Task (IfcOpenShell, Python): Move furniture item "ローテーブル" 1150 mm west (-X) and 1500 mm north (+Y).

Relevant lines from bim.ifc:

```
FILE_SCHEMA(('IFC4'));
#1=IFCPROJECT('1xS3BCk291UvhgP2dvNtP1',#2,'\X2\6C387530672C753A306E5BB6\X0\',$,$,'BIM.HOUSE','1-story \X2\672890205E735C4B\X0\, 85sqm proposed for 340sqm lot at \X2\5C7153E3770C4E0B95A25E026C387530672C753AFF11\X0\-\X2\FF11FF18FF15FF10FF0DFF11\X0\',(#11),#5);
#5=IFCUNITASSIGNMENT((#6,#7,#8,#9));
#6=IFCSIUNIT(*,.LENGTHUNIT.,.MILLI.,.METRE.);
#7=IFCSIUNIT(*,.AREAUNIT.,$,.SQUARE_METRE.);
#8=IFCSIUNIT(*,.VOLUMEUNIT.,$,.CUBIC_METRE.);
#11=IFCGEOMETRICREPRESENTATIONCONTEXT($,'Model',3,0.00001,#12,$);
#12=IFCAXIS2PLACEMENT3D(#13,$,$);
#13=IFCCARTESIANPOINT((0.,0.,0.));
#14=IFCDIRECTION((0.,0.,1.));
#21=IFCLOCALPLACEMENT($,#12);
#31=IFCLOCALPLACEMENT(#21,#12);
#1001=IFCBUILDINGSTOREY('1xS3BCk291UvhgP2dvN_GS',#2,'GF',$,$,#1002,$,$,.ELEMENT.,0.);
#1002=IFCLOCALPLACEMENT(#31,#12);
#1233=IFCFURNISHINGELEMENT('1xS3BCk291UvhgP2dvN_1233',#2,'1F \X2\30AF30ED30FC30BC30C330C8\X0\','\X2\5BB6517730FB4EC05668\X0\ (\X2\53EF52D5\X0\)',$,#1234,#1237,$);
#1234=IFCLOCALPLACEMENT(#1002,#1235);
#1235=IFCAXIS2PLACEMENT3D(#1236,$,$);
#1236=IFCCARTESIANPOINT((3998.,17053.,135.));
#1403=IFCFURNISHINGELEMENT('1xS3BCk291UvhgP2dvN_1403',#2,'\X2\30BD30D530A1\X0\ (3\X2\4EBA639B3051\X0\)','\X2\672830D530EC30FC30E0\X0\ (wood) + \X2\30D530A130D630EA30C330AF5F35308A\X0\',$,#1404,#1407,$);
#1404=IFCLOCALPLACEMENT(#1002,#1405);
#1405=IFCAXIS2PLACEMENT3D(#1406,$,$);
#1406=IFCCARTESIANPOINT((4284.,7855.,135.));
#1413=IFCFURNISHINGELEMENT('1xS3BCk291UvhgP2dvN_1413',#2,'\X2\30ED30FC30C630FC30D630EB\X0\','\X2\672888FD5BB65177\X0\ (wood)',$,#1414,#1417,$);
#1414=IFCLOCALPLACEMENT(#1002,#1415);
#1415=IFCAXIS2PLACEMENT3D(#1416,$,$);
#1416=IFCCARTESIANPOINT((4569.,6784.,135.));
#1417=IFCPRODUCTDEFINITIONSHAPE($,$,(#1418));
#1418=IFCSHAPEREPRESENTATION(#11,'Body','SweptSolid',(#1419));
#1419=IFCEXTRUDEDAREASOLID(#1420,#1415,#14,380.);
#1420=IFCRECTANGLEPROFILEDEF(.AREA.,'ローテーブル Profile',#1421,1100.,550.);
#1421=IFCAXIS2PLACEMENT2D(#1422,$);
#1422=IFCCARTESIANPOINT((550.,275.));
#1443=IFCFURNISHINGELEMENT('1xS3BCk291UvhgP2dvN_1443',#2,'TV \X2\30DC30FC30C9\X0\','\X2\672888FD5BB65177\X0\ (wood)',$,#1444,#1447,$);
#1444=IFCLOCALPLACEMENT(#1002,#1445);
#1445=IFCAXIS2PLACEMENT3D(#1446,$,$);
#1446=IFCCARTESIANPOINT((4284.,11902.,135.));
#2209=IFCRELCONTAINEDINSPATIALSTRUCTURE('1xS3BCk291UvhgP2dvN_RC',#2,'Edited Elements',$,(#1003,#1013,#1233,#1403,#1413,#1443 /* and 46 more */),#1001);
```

```python
import ifcopenshell
import ifcopenshell.api.geometry
import ifcopenshell.util.placement
import ifcopenshell.util.unit

model = ifcopenshell.open("bim.ifc")
unit_scale = ifcopenshell.util.unit.calculate_unit_scale(model)

item = model.by_guid("1xS3BCk291UvhgP2dvN_1413")
matrix = ifcopenshell.util.placement.get_local_placement(item.ObjectPlacement)
matrix[0, 3] -= 1.15 / unit_scale
matrix[1, 3] += 1.5 / unit_scale
ifcopenshell.api.geometry.edit_object_placement(model, product=item, matrix=matrix, is_si=False)

print(ifcopenshell.util.placement.get_local_placement(item.ObjectPlacement).round(3) + 0.0)

model.write("bim_v2.ifc")
```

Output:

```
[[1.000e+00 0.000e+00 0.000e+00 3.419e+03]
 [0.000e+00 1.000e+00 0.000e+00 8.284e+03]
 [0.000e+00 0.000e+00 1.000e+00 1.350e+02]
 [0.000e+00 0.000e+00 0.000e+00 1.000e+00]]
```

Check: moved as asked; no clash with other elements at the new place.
